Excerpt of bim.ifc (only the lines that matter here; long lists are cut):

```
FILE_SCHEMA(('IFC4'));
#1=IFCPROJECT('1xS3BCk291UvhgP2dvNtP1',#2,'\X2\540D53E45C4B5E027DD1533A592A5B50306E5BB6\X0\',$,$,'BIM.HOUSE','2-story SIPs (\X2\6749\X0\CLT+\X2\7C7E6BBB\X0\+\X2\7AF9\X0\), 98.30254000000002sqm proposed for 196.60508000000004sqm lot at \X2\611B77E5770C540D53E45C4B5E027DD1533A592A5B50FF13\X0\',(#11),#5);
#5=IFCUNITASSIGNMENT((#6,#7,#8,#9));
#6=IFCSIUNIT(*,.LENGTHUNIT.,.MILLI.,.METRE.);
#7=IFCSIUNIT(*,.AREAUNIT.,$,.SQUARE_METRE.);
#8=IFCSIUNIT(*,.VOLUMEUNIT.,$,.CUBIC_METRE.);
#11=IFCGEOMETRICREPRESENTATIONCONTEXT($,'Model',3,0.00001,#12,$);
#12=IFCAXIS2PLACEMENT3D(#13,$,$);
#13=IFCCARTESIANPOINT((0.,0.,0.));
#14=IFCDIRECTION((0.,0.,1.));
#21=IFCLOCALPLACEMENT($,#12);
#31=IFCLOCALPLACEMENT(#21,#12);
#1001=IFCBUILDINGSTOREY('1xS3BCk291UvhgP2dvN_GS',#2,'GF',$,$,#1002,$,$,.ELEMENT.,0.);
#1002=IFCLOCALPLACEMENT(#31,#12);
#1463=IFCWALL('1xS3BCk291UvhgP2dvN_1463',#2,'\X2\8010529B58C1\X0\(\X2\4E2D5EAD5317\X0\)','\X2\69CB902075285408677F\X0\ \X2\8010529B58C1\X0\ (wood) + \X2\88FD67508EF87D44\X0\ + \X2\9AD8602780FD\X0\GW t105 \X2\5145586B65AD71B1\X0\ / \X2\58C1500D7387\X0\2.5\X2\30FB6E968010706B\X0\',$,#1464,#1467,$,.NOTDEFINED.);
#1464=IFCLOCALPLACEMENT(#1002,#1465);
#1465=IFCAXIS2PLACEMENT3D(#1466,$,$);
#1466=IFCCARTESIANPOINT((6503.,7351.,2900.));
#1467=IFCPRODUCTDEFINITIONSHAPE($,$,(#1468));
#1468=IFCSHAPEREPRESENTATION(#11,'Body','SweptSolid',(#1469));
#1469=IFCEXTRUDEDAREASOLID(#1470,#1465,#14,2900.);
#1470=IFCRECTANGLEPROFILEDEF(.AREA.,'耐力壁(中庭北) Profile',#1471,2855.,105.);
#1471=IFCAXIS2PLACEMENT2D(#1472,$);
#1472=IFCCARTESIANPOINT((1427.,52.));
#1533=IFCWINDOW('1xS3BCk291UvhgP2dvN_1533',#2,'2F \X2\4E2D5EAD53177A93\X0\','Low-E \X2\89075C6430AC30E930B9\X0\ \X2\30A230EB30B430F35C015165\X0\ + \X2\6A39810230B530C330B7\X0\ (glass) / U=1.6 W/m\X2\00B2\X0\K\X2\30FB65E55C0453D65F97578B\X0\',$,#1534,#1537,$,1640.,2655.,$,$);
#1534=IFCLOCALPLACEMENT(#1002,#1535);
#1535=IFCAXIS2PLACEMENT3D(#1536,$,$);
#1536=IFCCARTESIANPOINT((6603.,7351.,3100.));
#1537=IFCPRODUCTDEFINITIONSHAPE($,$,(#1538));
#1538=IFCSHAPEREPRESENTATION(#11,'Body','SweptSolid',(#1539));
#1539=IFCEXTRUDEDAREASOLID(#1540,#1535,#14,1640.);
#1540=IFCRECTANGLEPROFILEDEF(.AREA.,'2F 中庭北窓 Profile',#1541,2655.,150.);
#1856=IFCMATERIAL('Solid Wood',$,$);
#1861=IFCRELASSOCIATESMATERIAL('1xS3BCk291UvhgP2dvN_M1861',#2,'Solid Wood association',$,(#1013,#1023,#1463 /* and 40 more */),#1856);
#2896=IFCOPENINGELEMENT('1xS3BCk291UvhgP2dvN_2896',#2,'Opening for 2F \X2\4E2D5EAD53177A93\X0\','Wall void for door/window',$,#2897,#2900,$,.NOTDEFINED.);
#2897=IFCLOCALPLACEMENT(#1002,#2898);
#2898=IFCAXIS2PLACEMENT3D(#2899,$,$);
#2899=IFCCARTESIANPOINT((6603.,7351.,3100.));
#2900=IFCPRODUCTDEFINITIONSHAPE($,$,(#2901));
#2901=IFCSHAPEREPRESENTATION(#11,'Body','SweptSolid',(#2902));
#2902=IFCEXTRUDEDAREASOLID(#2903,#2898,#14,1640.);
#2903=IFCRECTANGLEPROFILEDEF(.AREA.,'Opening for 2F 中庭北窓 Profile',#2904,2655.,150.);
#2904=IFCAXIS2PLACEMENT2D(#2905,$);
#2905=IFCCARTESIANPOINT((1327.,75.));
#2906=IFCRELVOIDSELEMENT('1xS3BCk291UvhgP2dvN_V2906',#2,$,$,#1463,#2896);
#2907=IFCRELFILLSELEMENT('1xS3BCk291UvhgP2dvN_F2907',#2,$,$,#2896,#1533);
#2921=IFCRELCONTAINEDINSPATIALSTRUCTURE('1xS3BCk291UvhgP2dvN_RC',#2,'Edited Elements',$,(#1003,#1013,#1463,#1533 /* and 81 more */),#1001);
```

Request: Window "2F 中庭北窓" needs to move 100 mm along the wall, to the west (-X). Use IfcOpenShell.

```python
import ifcopenshell
import ifcopenshell.api.geometry
import ifcopenshell.util.placement
import ifcopenshell.util.unit

model = ifcopenshell.open("bim.ifc")
unit_scale = ifcopenshell.util.unit.calculate_unit_scale(model)

window = model.by_guid("1xS3BCk291UvhgP2dvN_1533")
opening = window.FillsVoids[0].RelatingOpeningElement
wall = opening.VoidsElements[0].RelatingBuildingElement

wall_matrix = ifcopenshell.util.placement.get_local_placement(wall.ObjectPlacement)
shift = wall_matrix[:3, 0] * -0.1 / unit_scale
before = ifcopenshell.util.placement.get_local_placement(window.ObjectPlacement)[:3, 3].copy()

# The window is not placed relative to its opening, so move both.
for product in (opening, window):
    matrix = ifcopenshell.util.placement.get_local_placement(product.ObjectPlacement)
    matrix[:3, 3] += shift
    ifcopenshell.api.geometry.edit_object_placement(model, product=product, matrix=matrix, is_si=False)

after = ifcopenshell.util.placement.get_local_placement(window.ObjectPlacement)[:3, 3]
print("window moved by", (after - before).round(3) + 0.0)

model.write("bim_v2.ifc")
```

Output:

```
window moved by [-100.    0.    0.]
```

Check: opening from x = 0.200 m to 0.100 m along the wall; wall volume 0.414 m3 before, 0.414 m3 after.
